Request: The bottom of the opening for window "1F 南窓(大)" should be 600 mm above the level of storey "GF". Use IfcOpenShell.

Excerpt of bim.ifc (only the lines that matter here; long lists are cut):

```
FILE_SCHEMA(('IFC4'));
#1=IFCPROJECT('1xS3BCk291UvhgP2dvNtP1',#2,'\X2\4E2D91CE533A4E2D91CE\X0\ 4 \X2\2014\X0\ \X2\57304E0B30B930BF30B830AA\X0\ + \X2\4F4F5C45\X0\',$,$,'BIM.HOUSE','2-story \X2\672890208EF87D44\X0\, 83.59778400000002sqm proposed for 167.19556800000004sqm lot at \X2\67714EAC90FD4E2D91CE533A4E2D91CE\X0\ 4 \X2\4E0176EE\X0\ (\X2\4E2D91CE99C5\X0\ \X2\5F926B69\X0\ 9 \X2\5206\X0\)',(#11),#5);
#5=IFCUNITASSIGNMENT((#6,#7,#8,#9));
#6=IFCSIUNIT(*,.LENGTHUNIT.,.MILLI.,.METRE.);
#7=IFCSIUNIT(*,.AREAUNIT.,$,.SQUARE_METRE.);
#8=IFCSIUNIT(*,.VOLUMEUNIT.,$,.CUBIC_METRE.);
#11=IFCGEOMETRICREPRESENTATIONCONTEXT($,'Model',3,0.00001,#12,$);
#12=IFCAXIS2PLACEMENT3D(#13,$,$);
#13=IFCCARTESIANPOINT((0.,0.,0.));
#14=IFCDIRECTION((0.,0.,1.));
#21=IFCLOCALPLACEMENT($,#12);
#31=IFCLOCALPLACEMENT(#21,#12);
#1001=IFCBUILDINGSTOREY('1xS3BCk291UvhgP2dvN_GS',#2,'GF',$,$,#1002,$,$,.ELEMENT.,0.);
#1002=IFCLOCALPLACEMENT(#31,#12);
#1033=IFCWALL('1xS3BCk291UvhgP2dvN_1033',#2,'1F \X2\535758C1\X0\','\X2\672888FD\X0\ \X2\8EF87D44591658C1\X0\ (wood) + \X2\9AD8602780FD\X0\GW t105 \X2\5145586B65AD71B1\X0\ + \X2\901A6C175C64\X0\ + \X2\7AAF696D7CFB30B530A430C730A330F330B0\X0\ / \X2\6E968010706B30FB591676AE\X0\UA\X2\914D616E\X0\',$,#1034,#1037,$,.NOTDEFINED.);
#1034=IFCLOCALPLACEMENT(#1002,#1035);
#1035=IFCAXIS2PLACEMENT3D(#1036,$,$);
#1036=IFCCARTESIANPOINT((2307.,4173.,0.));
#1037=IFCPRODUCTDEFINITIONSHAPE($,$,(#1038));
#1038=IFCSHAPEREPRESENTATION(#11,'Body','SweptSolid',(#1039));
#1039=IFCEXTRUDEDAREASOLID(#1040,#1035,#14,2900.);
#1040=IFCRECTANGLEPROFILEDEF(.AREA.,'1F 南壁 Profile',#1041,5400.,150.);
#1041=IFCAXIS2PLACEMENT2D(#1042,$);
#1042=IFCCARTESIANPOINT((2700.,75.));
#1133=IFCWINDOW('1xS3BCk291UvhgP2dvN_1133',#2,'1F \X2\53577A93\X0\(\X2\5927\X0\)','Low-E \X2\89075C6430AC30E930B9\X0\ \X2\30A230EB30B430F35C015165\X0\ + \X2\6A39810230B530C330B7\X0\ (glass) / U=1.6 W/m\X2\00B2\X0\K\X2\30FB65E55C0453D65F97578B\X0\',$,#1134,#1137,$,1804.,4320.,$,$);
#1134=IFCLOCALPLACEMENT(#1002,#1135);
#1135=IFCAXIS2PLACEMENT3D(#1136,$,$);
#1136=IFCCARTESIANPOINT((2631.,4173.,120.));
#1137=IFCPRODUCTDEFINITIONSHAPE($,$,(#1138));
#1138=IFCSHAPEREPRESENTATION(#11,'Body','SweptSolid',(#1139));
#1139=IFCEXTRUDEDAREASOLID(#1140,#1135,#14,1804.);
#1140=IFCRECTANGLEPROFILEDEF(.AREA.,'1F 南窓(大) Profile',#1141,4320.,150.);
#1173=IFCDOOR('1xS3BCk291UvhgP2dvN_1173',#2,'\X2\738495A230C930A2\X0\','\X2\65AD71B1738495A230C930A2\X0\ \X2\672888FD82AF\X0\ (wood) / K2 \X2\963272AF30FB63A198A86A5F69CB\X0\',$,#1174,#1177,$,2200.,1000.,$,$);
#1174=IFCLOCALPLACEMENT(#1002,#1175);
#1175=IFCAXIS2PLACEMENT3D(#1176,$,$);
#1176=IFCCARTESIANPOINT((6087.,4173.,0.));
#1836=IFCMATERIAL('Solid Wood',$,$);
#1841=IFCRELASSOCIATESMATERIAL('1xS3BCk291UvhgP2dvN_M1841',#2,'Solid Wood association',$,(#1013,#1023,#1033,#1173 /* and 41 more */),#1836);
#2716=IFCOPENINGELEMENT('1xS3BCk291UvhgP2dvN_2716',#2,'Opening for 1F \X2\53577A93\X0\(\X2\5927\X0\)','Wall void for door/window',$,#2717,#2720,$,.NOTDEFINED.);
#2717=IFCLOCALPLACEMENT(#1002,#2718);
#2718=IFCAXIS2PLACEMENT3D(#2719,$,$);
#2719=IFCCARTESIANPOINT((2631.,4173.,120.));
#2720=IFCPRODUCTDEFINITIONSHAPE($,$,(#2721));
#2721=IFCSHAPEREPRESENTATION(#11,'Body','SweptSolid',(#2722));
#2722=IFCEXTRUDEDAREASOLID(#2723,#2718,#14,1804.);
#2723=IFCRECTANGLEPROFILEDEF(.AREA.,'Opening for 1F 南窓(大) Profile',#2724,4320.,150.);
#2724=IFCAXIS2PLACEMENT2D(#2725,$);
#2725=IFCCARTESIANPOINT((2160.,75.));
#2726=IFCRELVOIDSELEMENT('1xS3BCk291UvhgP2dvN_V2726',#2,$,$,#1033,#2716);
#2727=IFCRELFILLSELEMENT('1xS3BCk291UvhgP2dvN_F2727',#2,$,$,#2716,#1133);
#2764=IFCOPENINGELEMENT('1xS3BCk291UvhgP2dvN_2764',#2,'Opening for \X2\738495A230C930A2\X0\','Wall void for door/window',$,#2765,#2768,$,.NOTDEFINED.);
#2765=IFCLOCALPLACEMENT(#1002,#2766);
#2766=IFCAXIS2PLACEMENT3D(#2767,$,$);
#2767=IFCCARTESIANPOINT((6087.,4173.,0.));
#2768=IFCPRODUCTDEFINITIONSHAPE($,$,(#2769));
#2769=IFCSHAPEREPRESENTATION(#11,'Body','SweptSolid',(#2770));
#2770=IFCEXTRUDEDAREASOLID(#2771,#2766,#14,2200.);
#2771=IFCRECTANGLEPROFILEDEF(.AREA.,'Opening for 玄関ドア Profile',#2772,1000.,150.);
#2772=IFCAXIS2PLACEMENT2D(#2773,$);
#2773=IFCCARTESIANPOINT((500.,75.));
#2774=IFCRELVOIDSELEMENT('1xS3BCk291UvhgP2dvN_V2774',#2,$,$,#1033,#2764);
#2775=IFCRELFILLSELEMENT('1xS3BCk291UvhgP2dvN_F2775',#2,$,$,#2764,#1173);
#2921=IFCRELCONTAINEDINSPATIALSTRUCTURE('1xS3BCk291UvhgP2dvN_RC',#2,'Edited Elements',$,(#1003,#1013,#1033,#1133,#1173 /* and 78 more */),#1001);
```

```python
import numpy as np
import ifcopenshell
import ifcopenshell.api.geometry
import ifcopenshell.geom
import ifcopenshell.util.element
import ifcopenshell.util.placement
import ifcopenshell.util.shape
import ifcopenshell.util.unit

model = ifcopenshell.open("bim.ifc")
unit_scale = ifcopenshell.util.unit.calculate_unit_scale(model)

window = model.by_guid("1xS3BCk291UvhgP2dvN_1133")
opening = window.FillsVoids[0].RelatingOpeningElement
storey = ifcopenshell.util.element.get_container(window, ifc_class="IfcBuildingStorey")
level = ifcopenshell.util.placement.get_local_placement(storey.ObjectPlacement)[2, 3]

# The opening's origin need not be at the sill, so measure its lowest point.
shape = ifcopenshell.geom.create_shape(ifcopenshell.geom.settings(), opening)
bottom = ifcopenshell.util.shape.get_shape_bottom_elevation(shape, shape.geometry) / unit_scale
dz = level + 0.6 / unit_scale - bottom

shift = np.array([0.0, 0.0, dz])
# The window is not placed relative to its opening, so move both.
for product in (opening, window):
    matrix = ifcopenshell.util.placement.get_local_placement(product.ObjectPlacement)
    matrix[:3, 3] += shift
    ifcopenshell.api.geometry.edit_object_placement(model, product=product, matrix=matrix, is_si=False)

print(f"moved by {dz * unit_scale:+.3f} m")

model.write("bim_rev.ifc")
```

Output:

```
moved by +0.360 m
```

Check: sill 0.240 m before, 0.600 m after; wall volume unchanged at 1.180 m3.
